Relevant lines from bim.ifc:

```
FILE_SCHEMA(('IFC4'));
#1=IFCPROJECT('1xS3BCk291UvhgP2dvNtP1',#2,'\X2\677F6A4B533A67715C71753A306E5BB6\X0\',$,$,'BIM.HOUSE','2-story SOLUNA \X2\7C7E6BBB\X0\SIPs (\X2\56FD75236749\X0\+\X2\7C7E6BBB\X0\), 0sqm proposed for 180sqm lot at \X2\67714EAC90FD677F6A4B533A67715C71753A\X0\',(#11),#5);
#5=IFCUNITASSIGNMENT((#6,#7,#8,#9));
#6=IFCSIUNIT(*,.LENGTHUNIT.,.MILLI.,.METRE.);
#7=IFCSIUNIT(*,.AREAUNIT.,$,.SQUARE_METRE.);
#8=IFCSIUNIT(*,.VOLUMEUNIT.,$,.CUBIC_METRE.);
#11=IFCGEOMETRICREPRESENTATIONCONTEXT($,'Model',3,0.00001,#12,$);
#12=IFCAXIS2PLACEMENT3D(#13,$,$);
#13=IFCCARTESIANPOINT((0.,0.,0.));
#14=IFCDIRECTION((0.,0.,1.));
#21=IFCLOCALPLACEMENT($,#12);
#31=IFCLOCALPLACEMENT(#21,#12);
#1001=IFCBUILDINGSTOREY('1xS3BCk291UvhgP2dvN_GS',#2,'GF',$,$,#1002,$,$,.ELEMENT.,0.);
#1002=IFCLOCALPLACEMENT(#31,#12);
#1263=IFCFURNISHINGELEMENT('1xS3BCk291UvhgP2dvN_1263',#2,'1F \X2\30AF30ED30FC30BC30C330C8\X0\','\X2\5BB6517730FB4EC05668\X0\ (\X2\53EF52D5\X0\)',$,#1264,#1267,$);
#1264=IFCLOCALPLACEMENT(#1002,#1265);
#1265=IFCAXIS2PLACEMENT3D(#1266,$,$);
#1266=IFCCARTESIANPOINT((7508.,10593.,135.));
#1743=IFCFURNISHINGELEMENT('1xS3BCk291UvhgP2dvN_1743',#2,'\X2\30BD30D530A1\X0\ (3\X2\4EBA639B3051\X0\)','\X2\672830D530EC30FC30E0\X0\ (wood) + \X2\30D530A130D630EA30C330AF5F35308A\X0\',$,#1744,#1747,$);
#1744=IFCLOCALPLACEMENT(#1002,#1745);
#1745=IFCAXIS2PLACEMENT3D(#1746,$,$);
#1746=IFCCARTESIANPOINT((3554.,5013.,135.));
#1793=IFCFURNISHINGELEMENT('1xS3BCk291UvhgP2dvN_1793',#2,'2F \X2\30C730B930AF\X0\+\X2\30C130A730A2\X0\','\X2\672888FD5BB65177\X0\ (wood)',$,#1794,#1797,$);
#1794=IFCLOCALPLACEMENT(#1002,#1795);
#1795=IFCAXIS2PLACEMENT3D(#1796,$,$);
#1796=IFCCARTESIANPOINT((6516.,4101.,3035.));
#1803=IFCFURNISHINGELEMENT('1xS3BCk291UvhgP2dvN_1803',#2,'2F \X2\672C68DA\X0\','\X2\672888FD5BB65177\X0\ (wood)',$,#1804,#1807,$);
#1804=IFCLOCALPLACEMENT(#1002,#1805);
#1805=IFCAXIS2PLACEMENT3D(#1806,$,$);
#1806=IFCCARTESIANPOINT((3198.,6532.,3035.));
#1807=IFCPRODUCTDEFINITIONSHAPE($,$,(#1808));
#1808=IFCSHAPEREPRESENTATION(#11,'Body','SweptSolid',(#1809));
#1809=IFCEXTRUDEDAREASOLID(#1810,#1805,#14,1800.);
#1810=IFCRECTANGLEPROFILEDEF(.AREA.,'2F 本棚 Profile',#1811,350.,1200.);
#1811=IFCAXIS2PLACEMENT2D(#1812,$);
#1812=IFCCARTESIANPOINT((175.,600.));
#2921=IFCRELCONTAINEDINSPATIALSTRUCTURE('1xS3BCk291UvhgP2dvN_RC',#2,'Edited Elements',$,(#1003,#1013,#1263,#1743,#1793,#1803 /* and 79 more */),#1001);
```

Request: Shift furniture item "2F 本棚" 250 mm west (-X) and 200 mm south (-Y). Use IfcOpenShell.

```python
import ifcopenshell
import ifcopenshell.api.geometry
import ifcopenshell.util.placement

model = ifcopenshell.open("bim.ifc")

item = model.by_id(1803)
matrix = ifcopenshell.util.placement.get_local_placement(item.ObjectPlacement)
matrix[0, 3] -= 250.0
matrix[1, 3] -= 200.0
ifcopenshell.api.geometry.edit_object_placement(model, product=item, matrix=matrix, is_si=False)

print(ifcopenshell.util.placement.get_local_placement(item.ObjectPlacement).round(3) + 0.0)

model.write("bim_edited.ifc")
```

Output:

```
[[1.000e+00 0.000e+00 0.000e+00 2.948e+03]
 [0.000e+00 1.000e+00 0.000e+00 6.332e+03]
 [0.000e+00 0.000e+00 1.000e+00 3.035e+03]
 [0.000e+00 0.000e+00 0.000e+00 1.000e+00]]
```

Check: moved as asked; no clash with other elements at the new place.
